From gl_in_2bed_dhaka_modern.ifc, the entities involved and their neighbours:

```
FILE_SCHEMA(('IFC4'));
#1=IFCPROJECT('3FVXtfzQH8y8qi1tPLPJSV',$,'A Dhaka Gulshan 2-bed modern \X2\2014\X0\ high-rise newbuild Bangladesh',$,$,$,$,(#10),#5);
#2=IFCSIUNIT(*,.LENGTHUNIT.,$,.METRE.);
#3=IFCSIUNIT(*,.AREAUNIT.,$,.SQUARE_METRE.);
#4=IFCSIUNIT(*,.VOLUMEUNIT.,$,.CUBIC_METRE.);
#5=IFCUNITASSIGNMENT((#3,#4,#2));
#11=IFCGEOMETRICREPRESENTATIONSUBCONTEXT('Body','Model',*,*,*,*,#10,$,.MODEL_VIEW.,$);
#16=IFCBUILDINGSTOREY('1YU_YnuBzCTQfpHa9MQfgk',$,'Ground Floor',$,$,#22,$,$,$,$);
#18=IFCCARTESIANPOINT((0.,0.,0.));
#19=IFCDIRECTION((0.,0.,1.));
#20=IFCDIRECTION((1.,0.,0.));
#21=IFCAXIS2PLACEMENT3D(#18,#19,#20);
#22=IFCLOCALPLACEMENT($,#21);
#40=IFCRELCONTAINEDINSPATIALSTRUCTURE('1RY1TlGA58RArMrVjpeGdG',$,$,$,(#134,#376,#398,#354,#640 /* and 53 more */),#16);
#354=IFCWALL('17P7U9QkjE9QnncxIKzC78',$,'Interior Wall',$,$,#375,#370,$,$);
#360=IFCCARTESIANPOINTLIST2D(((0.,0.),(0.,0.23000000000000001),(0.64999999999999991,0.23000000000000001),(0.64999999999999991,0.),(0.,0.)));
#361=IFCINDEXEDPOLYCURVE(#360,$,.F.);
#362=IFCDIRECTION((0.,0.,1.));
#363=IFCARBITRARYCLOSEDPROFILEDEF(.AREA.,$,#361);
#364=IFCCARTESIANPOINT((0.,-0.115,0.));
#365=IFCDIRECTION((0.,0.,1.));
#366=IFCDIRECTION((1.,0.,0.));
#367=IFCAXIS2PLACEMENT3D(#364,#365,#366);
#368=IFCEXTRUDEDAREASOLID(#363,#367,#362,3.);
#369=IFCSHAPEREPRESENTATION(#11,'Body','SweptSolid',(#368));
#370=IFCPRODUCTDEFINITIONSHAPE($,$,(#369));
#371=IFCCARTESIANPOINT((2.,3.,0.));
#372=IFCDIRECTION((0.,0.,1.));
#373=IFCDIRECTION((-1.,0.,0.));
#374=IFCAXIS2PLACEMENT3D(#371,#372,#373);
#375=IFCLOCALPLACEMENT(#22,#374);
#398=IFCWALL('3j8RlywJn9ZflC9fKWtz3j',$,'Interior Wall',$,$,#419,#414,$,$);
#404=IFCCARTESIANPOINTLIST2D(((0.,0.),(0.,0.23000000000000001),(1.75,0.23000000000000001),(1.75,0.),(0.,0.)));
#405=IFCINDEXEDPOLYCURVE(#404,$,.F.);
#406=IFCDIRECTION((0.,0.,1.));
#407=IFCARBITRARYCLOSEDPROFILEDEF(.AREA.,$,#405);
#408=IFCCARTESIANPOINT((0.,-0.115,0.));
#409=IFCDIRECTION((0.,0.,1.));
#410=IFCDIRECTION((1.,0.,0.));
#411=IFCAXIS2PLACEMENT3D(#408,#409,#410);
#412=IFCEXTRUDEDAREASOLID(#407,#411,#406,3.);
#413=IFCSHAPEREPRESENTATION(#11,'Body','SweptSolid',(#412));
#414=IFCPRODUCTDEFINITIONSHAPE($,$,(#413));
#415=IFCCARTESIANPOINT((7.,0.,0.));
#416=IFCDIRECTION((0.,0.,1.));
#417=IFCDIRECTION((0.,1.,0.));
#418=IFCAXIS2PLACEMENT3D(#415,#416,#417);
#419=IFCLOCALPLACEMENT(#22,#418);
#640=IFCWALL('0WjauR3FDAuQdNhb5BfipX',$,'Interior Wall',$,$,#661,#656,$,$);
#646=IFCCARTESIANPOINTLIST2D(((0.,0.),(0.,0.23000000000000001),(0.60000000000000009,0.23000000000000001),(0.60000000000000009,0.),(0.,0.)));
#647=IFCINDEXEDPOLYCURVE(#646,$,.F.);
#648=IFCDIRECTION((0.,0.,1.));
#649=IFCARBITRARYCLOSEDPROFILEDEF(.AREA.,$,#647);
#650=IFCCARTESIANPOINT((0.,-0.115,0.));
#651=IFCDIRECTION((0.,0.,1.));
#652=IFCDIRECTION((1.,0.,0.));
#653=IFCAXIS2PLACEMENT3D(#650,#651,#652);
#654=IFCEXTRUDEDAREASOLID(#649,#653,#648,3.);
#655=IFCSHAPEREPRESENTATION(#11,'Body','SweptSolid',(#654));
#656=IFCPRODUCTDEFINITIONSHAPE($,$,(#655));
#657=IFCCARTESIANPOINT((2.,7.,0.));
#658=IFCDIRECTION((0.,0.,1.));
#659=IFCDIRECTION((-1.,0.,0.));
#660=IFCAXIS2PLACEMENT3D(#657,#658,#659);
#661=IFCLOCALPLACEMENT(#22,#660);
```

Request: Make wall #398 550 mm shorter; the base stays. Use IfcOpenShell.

```python
import ifcopenshell
import ifcopenshell.geom
import ifcopenshell.util.representation
import ifcopenshell.util.shape
import ifcopenshell.util.unit

model = ifcopenshell.open("gl_in_2bed_dhaka_modern.ifc")
unit_scale = ifcopenshell.util.unit.calculate_unit_scale(model)
settings = ifcopenshell.geom.settings()


def volume(element):
    """Net volume in cubic metres, openings subtracted."""
    shape = ifcopenshell.geom.create_shape(settings, element)
    return ifcopenshell.util.shape.get_volume(shape.geometry)


wall = model.by_guid("3j8RlywJn9ZflC9fKWtz3j")
before = volume(wall)

body = ifcopenshell.util.representation.get_representation(wall, "Model", "Body")
solid = body.Items[0]
old_height = solid.Depth
solid.Depth -= 0.55 / unit_scale
after = volume(wall)

print(f"height {old_height:g} -> {solid.Depth:g}, volume {before:.3f} -> {after:.3f} m3")

model.write("gl_in_2bed_dhaka_modern_updated.ifc")
```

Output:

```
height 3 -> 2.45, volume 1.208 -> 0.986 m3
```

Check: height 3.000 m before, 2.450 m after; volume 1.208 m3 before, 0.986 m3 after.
